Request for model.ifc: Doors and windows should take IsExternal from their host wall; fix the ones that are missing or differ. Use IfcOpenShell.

First a look at what the model holds.

```python
import ifcopenshell
import ifcopenshell.util.element

model = ifcopenshell.open("model.ifc")
print(model.schema)
seen = {}
for e in model.by_type("IfcDoor") + model.by_type("IfcWindow"):
    if not e.FillsVoids:
        continue
    host = e.FillsVoids[0].RelatingOpeningElement.VoidsElements[0].RelatingBuildingElement
    own = ifcopenshell.util.element.get_pset(e, f"Pset_{e.is_a()[3:].removesuffix('StandardCase')}Common", "IsExternal")
    wall = ifcopenshell.util.element.get_pset(host, "Pset_WallCommon", "IsExternal")
    seen[e.is_a(), own, wall] = seen.get((e.is_a(), own, wall), 0) + 1
for (cls, own, wall), count in sorted(seen.items(), key=str):
    print(count, cls, "IsExternal:", own, "| host wall:", wall)
```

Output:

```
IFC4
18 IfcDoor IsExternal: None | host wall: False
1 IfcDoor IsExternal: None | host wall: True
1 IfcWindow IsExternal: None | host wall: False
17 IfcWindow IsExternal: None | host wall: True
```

```python
import ifcopenshell
import ifcopenshell.api.pset
import ifcopenshell.util.element

model = ifcopenshell.open("model.ifc")

count = 0
for ifc_class, pset_name in (("IfcDoor", "Pset_DoorCommon"), ("IfcWindow", "Pset_WindowCommon")):
    for e in model.by_type(ifc_class):
        if not e.FillsVoids:
            continue
        host = e.FillsVoids[0].RelatingOpeningElement.VoidsElements[0].RelatingBuildingElement
        external = ifcopenshell.util.element.get_pset(host, "Pset_WallCommon", "IsExternal")
        if external is None or ifcopenshell.util.element.get_pset(e, pset_name, "IsExternal") == external:
            continue
        pset = ifcopenshell.api.pset.add_pset(model, product=e, name=pset_name)
        ifcopenshell.api.pset.edit_pset(model, pset=pset, properties={"IsExternal": external})
        count += 1

print(count, "updated")

model.write("model_rev.ifc")
```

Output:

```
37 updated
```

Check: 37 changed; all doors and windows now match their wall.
